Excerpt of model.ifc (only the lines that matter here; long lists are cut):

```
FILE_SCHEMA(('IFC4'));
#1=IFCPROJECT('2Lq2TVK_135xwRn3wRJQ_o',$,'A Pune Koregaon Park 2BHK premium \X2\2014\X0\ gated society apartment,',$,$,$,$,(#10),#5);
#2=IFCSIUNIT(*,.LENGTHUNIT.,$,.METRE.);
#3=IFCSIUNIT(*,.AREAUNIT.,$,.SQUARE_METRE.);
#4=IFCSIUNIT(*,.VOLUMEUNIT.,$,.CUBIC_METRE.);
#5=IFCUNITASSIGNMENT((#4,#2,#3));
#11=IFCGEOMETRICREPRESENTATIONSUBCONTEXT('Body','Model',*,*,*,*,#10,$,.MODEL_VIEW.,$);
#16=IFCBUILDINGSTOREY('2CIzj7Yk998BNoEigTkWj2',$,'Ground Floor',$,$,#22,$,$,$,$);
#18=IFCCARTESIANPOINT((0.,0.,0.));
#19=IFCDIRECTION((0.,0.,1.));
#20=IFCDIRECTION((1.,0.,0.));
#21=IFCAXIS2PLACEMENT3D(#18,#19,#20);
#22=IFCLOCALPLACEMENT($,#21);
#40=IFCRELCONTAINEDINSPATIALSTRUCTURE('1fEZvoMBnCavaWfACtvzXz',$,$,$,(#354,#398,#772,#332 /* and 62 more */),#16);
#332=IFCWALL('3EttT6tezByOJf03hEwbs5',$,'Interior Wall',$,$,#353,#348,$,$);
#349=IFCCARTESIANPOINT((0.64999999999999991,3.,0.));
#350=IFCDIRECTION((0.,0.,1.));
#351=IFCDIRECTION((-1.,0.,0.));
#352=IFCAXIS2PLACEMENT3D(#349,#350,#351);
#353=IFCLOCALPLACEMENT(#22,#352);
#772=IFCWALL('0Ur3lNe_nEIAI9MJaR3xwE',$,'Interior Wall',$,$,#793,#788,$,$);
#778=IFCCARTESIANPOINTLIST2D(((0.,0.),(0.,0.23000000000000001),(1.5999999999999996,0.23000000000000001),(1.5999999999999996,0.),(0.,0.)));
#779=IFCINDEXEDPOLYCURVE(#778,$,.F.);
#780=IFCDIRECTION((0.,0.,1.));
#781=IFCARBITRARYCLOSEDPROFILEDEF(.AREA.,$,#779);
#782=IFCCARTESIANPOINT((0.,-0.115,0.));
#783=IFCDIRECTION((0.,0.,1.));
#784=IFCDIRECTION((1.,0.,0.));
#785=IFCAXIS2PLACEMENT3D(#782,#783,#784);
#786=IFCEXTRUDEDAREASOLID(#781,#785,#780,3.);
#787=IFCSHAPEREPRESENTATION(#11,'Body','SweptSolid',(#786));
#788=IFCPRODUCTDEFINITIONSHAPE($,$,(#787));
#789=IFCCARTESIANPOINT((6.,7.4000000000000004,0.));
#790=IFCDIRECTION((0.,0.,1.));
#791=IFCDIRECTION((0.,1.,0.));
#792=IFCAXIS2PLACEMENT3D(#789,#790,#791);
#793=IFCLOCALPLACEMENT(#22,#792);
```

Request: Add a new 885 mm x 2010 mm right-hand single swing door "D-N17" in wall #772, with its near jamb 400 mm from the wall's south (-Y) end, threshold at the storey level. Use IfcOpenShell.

```python
import numpy as np
import ifcopenshell
import ifcopenshell.api.feature
import ifcopenshell.api.geometry
import ifcopenshell.api.root
import ifcopenshell.api.spatial
import ifcopenshell.geom
import ifcopenshell.util.element
import ifcopenshell.util.placement
import ifcopenshell.util.representation
import ifcopenshell.util.shape
import ifcopenshell.util.unit

model = ifcopenshell.open("model.ifc")
unit_scale = ifcopenshell.util.unit.calculate_unit_scale(model)
settings = ifcopenshell.geom.settings()


def volume(element):
    """Net volume in cubic metres, openings subtracted."""
    shape = ifcopenshell.geom.create_shape(settings, element)
    return ifcopenshell.util.shape.get_volume(shape.geometry)


wall = model.by_guid("0Ur3lNe_nEIAI9MJaR3xwE")
storey = ifcopenshell.util.element.get_container(wall, ifc_class="IfcBuildingStorey")
context = ifcopenshell.util.representation.get_context(model, "Model", "Body", "MODEL_VIEW")
before = volume(wall)

width, height, from_end, sill = 0.885, 2.01, 0.4, 0.0  # metres

# The wall runs along its own X axis, and the end named is its -X end.
wall_shape = ifcopenshell.geom.create_shape(settings, wall)
x, y, z = ifcopenshell.util.shape.get_vertices(wall_shape.geometry).T
start = x.min() + from_end
face, thickness = float(y.min()), float(y.max() - y.min())
wall_matrix = ifcopenshell.util.placement.get_local_placement(wall.ObjectPlacement)
level = ifcopenshell.util.placement.get_local_placement(storey.ObjectPlacement)[2, 3]


def in_wall(x, y):
    """Placement at x, y metres in the wall's axes, at sill height."""
    matrix = wall_matrix.copy()
    matrix[:, 3] = wall_matrix @ np.array([x / unit_scale, y / unit_scale, 0.0, 1.0])
    matrix[2, 3] = level + sill / unit_scale
    return matrix


# Opening: a box that overshoots both wall faces by 50 mm.
opening = ifcopenshell.api.root.create_entity(model, ifc_class="IfcOpeningElement", predefined_type="OPENING")
box = ifcopenshell.api.geometry.add_wall_representation(
    model, context=context, length=width, height=height, thickness=thickness + 0.1
)
ifcopenshell.api.geometry.assign_representation(model, product=opening, representation=box)
ifcopenshell.api.geometry.edit_object_placement(model, product=opening, matrix=in_wall(start, face - 0.05), is_si=False)
ifcopenshell.api.feature.add_feature(model, feature=opening, element=wall)

door = ifcopenshell.api.root.create_entity(model, ifc_class="IfcDoor", name="D-N17", predefined_type="DOOR")
door.OverallWidth, door.OverallHeight = width / unit_scale, height / unit_scale
door.OperationType = "SINGLE_SWING_RIGHT"
body = ifcopenshell.api.geometry.add_door_representation(
    model,
    context=context,
    overall_width=door.OverallWidth,
    overall_height=door.OverallHeight,
    operation_type="SINGLE_SWING_RIGHT",
    lining_properties={"LiningDepth": thickness / unit_scale, "ThresholdDepth": thickness / unit_scale},
)
ifcopenshell.api.geometry.assign_representation(model, product=door, representation=body)
ifcopenshell.api.spatial.assign_container(model, products=[door], relating_structure=storey)
ifcopenshell.api.feature.add_filling(model, opening=opening, element=door)

# The lining spans the wall, so the door starts at the wall face.
ifcopenshell.api.geometry.edit_object_placement(model, product=door, matrix=in_wall(start, face), is_si=False)

after = volume(wall)

print(f"wall volume {before:.3f} -> {after:.3f} m3")

model.write("model-out.ifc")
```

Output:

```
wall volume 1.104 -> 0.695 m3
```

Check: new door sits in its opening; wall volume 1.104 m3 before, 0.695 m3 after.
